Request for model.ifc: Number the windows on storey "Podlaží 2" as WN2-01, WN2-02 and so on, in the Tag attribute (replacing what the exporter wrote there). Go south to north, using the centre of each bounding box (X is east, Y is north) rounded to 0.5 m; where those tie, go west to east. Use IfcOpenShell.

First a look at what the model holds.

```python
import ifcopenshell
import ifcopenshell.util.element
import ifcopenshell.util.placement

model = ifcopenshell.open("model.ifc")
print(model.schema)
storey = next(s for s in model.by_type("IfcBuildingStorey") if s.Name == "Podlaží 2")
windows = [e for e in ifcopenshell.util.element.get_decomposition(storey) if e.is_a("IfcWindow")]
for e in sorted(windows, key=lambda e: e.id()):
    origin = ifcopenshell.util.placement.get_local_placement(e.ObjectPlacement)[:3, 3]
    print(e.id(), e.Tag, e.Name, origin.round(2) + 0.0, sep=" | ")
```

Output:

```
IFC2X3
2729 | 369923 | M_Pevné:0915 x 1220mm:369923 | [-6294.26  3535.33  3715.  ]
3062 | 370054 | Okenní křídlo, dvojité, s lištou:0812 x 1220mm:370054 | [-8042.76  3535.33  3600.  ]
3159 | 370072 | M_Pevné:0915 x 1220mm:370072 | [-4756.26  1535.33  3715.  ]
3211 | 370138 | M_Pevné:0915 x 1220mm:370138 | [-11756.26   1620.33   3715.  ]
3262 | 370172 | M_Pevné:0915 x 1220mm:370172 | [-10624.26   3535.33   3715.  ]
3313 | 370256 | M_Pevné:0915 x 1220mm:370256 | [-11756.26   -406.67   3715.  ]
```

```python
import ifcopenshell
import ifcopenshell.geom
import ifcopenshell.util.element
import ifcopenshell.util.shape

model = ifcopenshell.open("model.ifc")
settings = ifcopenshell.geom.settings()
settings.set("use-world-coords", True)


def centre(element):
    shape = ifcopenshell.geom.create_shape(settings, element)
    return ifcopenshell.util.shape.get_bbox_centroid(shape.geometry)


storey = next(s for s in model.by_type("IfcBuildingStorey") if s.Name == "Podlaží 2")
windows = [e for e in ifcopenshell.util.element.get_decomposition(storey) if e.is_a("IfcWindow")]

# Insertion points can sit at a corner or the storey origin, so sort by the geometry (in metres).
centres = {e: centre(e) for e in windows}
windows.sort(key=lambda e: (round(centres[e][1] / 0.5), centres[e][0]))

for i, e in enumerate(windows, start=1):
    number = f"WN2-{i:02d}"
    e.Tag = number
    print(e.id(), number)

model.write("model_rev.ifc")
```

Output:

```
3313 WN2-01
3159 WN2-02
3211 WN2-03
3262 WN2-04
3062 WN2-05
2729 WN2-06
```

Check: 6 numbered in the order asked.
